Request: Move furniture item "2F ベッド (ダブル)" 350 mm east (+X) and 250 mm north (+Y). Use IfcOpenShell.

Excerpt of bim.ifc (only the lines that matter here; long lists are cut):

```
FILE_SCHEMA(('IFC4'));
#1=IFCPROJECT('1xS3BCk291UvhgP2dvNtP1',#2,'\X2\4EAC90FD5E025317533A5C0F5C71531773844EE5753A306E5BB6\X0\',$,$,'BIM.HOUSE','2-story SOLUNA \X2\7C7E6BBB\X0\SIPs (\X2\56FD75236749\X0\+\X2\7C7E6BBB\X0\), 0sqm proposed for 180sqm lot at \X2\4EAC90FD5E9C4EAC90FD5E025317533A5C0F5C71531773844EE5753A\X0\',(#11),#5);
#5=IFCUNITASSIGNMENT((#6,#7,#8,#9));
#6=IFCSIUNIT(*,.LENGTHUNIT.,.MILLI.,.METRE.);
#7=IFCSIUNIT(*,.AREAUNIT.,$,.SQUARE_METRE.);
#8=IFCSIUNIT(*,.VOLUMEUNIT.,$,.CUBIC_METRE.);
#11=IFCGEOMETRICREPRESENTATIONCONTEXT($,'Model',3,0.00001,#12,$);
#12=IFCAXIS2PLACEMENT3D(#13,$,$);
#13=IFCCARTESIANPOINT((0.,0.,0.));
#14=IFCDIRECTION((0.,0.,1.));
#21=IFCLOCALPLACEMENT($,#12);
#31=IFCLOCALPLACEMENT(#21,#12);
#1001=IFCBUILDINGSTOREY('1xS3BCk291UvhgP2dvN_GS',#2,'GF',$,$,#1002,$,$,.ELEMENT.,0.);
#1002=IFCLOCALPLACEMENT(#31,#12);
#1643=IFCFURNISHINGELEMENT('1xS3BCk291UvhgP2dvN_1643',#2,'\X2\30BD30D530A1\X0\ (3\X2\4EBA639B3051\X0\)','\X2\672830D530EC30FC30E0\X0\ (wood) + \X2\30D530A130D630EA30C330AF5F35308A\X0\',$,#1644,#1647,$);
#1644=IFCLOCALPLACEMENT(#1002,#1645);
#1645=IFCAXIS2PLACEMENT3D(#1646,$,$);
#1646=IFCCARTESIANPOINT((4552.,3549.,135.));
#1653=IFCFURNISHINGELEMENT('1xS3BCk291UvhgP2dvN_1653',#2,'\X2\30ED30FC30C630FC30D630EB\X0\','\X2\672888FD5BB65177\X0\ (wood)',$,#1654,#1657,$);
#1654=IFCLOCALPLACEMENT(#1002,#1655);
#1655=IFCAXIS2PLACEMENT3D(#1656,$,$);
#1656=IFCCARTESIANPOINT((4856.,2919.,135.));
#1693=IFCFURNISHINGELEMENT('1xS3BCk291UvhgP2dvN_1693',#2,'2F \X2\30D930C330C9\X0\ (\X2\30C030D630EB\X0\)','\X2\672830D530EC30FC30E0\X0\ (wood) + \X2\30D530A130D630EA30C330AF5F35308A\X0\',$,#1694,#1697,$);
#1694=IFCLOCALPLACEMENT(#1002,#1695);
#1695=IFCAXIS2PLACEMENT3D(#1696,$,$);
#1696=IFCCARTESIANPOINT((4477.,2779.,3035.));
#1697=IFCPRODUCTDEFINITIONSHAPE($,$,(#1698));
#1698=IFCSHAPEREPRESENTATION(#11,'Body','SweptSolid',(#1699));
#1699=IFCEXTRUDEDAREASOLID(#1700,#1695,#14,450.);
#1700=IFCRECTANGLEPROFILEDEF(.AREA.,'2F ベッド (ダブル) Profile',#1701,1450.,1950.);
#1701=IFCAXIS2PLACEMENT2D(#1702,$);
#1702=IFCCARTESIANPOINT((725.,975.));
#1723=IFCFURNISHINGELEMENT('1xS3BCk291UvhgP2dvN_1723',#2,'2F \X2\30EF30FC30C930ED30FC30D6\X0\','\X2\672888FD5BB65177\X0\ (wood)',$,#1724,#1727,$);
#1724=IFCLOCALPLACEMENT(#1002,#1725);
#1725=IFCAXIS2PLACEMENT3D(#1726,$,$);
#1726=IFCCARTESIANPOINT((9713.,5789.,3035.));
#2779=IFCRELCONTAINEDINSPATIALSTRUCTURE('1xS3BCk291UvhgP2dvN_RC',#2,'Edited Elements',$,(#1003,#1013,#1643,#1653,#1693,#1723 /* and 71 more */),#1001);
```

```python
import ifcopenshell
import ifcopenshell.api.geometry
import ifcopenshell.util.placement

model = ifcopenshell.open("bim.ifc")

item = model.by_guid("1xS3BCk291UvhgP2dvN_1693")
matrix = ifcopenshell.util.placement.get_local_placement(item.ObjectPlacement)
matrix[0, 3] += 350.0
matrix[1, 3] += 250.0
ifcopenshell.api.geometry.edit_object_placement(model, product=item, matrix=matrix, is_si=False)

print(ifcopenshell.util.placement.get_local_placement(item.ObjectPlacement).round(3) + 0.0)

model.write("bim-out.ifc")
```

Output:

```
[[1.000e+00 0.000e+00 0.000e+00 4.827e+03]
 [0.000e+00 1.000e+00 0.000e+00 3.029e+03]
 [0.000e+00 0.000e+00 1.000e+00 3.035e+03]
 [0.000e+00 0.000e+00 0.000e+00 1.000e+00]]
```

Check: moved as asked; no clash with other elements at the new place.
